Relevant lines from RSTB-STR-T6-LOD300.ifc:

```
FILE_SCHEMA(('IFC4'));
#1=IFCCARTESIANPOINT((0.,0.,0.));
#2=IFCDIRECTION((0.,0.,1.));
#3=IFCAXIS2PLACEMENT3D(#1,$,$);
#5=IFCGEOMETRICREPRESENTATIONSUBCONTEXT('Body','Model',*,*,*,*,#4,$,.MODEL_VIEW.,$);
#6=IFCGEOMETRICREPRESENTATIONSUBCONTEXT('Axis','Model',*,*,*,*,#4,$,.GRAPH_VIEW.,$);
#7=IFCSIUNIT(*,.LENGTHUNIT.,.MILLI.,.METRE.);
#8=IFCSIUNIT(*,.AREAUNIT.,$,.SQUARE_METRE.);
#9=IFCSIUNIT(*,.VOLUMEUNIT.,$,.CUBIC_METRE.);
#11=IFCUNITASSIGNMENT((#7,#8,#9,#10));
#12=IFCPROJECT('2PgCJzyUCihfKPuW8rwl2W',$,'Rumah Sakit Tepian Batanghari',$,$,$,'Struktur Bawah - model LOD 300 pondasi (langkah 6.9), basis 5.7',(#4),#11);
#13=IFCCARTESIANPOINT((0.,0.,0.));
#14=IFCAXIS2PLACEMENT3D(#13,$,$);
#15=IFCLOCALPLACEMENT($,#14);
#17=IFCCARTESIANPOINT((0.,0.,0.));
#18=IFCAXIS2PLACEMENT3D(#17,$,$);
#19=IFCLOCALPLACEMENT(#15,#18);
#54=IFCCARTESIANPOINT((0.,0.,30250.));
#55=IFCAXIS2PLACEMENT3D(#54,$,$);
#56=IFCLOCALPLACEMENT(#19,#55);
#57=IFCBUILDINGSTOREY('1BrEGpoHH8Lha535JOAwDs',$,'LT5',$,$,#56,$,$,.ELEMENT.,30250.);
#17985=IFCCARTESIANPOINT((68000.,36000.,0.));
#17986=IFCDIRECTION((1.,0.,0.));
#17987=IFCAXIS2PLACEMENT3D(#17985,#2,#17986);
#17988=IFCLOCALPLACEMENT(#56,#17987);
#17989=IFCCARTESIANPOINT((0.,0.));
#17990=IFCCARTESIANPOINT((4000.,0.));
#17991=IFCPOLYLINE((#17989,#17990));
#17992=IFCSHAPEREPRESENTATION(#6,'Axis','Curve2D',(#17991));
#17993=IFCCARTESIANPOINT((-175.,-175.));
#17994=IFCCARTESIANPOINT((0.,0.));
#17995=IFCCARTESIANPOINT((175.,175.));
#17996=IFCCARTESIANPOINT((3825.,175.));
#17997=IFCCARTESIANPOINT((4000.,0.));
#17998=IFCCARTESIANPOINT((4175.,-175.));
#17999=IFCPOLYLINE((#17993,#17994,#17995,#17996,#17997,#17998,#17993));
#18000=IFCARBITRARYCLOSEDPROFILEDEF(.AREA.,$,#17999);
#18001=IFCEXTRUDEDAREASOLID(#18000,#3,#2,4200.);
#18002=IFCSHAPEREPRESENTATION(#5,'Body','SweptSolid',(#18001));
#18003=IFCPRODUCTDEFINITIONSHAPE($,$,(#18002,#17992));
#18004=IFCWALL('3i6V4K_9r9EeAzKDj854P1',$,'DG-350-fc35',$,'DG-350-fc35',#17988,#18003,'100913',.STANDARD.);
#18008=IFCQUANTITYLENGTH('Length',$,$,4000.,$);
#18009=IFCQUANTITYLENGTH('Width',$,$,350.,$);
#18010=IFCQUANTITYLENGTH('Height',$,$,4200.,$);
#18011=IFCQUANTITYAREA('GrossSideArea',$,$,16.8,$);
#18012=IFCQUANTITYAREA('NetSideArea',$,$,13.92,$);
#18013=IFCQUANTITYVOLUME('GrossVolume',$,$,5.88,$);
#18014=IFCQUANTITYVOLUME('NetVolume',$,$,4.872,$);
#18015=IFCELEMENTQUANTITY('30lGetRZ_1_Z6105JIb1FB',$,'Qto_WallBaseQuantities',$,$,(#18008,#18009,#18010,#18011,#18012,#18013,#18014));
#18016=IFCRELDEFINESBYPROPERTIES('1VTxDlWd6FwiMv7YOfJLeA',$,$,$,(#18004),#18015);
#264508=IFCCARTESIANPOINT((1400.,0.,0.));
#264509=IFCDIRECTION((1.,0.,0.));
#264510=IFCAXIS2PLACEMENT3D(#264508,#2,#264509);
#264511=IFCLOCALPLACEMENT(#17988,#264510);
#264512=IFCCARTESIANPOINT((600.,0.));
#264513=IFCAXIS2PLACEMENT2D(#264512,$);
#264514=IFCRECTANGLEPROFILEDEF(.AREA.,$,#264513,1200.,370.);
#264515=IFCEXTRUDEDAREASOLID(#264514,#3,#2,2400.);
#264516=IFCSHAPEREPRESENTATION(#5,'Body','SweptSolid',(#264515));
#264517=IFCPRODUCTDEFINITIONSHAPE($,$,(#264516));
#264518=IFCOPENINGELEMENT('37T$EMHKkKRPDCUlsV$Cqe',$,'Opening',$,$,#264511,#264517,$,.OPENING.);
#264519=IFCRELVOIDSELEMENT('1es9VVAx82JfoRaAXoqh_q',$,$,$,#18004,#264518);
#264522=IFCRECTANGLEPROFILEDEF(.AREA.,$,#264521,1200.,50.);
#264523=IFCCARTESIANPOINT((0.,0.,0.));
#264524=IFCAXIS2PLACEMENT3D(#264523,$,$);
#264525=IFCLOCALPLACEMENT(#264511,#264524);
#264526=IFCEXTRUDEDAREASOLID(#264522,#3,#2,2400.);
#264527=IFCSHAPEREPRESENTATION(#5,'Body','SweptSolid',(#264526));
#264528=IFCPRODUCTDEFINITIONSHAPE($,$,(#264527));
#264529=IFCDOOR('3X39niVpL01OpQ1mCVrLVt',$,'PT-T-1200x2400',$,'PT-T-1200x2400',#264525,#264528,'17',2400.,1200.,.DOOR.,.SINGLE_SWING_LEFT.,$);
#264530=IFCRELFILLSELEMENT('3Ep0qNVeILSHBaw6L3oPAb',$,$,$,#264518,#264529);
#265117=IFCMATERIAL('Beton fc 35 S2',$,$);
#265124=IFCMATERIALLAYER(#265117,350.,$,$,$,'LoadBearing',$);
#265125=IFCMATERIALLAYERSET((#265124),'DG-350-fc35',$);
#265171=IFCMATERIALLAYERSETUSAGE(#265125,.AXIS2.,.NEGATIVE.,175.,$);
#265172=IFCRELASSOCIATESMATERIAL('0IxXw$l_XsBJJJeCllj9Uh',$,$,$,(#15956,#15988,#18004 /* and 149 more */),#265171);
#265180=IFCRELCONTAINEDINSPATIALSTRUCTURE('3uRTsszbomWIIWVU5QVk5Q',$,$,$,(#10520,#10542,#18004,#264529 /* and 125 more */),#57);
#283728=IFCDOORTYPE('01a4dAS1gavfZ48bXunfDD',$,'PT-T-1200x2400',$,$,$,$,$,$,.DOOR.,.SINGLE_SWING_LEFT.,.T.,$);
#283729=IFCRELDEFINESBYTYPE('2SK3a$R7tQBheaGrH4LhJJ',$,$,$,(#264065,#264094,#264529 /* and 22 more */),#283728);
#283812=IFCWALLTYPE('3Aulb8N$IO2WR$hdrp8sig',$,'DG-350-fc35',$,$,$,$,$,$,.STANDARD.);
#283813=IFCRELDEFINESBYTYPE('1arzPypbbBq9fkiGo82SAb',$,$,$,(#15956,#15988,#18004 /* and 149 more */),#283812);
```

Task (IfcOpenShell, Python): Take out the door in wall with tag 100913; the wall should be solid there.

```python
import ifcopenshell
import ifcopenshell.api.feature
import ifcopenshell.api.pset
import ifcopenshell.api.root
import ifcopenshell.geom
import ifcopenshell.util.element
import ifcopenshell.util.shape
import ifcopenshell.util.unit

model = ifcopenshell.open("RSTB-STR-T6-LOD300.ifc")
area_scale = ifcopenshell.util.unit.calculate_unit_scale(model, "AREAUNIT")
volume_scale = ifcopenshell.util.unit.calculate_unit_scale(model, "VOLUMEUNIT")
settings = ifcopenshell.geom.settings()


def volume(element):
    """Net volume in cubic metres, openings subtracted."""
    shape = ifcopenshell.geom.create_shape(settings, element)
    return ifcopenshell.util.shape.get_volume(shape.geometry)


door = model.by_id(264529)
opening = door.FillsVoids[0].RelatingOpeningElement
wall = opening.VoidsElements[0].RelatingBuildingElement
before = volume(wall)

ifcopenshell.api.root.remove_product(model, product=door)
ifcopenshell.api.feature.remove_feature(model, feature=opening)

after = volume(wall)
thickness = 0.35  # wall thickness in metres

# Update the wall's stored quantities.
qto = model.by_id(ifcopenshell.util.element.get_pset(wall, "Qto_WallBaseQuantities", should_inherit=False)["id"])
ifcopenshell.api.pset.edit_qto(model, qto=qto, properties={
    "NetSideArea": after / thickness / area_scale,
    "NetVolume": after / volume_scale,
})

print(f"wall volume {before:.3f} -> {after:.3f} m3")

model.write("RSTB-STR-T6-LOD300_updated.ifc")
```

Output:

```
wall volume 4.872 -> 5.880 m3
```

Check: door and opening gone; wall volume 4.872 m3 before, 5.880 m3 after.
